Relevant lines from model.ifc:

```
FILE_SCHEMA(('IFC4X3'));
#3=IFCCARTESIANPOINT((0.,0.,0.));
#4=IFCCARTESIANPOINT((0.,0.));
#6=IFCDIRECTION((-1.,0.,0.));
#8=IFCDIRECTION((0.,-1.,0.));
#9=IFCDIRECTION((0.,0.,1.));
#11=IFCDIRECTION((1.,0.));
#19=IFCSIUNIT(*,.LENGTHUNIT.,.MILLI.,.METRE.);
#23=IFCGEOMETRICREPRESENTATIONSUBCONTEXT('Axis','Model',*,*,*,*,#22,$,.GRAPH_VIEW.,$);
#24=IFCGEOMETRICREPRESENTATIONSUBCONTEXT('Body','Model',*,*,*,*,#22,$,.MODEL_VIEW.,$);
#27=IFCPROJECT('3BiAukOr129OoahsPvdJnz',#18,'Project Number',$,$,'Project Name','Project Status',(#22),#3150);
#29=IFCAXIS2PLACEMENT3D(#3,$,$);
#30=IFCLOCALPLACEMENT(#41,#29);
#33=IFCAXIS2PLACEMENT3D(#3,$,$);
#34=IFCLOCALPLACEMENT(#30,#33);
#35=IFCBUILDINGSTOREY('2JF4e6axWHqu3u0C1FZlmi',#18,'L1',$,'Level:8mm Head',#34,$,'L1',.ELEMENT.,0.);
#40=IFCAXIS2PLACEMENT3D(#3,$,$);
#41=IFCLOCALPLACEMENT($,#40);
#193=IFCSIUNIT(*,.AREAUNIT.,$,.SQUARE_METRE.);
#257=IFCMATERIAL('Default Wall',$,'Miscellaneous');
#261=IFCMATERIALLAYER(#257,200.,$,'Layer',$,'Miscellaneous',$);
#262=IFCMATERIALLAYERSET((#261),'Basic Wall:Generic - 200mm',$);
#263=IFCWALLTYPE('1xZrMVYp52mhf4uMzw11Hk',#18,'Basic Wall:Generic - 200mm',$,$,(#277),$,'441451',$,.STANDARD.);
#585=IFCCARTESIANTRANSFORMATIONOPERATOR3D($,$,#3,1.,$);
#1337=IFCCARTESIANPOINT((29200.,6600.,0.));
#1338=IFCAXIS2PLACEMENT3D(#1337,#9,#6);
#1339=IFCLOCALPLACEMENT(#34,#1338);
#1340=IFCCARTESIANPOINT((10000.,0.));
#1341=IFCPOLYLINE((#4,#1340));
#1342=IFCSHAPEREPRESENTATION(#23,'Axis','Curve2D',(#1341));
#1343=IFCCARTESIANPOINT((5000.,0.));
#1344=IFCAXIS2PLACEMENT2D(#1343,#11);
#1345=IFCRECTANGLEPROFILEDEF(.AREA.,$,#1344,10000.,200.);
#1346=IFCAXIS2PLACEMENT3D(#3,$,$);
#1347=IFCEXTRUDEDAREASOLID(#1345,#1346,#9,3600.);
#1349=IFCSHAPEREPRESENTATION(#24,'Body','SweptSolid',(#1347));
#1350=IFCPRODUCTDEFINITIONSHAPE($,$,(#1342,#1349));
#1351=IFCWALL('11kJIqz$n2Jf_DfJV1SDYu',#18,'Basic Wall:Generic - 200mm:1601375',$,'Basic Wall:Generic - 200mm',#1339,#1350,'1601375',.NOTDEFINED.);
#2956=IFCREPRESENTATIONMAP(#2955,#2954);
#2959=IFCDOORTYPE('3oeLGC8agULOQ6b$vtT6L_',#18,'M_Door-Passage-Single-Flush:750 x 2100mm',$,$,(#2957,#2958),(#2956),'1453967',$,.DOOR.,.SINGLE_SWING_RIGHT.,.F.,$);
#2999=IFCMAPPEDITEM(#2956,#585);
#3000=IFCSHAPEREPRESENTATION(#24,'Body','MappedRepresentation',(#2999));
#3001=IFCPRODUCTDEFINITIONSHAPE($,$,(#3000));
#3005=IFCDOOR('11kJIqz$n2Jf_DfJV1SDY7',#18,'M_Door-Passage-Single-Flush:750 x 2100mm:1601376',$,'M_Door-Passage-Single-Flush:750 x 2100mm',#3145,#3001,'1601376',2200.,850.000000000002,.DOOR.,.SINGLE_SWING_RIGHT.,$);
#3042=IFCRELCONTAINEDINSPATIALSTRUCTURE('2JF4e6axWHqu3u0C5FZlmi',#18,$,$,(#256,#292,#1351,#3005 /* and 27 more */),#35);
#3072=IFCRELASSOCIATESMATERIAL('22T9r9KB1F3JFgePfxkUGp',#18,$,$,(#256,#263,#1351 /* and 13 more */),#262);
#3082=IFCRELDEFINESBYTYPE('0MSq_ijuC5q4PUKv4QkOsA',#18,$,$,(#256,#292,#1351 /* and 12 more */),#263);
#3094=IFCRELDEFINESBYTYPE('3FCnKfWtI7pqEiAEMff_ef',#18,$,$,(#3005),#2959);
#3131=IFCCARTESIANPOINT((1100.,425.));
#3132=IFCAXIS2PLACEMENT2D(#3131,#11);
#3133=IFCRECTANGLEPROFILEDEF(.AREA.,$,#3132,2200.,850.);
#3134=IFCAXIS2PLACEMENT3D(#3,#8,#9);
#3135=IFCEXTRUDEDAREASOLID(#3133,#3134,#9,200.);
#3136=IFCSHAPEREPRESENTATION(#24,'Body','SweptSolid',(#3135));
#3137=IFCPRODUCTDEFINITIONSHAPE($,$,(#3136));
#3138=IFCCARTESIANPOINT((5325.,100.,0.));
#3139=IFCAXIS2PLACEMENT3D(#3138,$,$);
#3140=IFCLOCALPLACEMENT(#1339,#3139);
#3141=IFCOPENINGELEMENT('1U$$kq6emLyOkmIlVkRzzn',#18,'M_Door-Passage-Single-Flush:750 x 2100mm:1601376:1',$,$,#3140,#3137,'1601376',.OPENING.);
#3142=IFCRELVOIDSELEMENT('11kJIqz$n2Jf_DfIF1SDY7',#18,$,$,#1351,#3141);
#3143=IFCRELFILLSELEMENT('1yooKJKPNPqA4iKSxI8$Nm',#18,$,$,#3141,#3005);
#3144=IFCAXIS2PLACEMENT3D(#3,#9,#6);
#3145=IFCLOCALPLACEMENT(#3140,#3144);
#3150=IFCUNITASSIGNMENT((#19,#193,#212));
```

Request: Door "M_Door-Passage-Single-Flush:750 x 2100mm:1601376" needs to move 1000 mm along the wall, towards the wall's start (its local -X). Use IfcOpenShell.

```python
import ifcopenshell
import ifcopenshell.api.geometry
import ifcopenshell.util.placement

model = ifcopenshell.open("model.ifc")

door = model.by_guid("11kJIqz$n2Jf_DfJV1SDY7")
opening = door.FillsVoids[0].RelatingOpeningElement
wall = opening.VoidsElements[0].RelatingBuildingElement

wall_matrix = ifcopenshell.util.placement.get_local_placement(wall.ObjectPlacement)
shift = wall_matrix[:3, 0] * -1000.0
before = ifcopenshell.util.placement.get_local_placement(door.ObjectPlacement)[:3, 3].copy()

# The door is placed relative to its opening, so it follows when the opening moves.
matrix = ifcopenshell.util.placement.get_local_placement(opening.ObjectPlacement)
matrix[:3, 3] += shift
ifcopenshell.api.geometry.edit_object_placement(
    model, product=opening, matrix=matrix, is_si=False, should_transform_children=True
)

after = ifcopenshell.util.placement.get_local_placement(door.ObjectPlacement)[:3, 3]
print("door moved by", (after - before).round(3) + 0.0)

model.write("model_v2.ifc")
```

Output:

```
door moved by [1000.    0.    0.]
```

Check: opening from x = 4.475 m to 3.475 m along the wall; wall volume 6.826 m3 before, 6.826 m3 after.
